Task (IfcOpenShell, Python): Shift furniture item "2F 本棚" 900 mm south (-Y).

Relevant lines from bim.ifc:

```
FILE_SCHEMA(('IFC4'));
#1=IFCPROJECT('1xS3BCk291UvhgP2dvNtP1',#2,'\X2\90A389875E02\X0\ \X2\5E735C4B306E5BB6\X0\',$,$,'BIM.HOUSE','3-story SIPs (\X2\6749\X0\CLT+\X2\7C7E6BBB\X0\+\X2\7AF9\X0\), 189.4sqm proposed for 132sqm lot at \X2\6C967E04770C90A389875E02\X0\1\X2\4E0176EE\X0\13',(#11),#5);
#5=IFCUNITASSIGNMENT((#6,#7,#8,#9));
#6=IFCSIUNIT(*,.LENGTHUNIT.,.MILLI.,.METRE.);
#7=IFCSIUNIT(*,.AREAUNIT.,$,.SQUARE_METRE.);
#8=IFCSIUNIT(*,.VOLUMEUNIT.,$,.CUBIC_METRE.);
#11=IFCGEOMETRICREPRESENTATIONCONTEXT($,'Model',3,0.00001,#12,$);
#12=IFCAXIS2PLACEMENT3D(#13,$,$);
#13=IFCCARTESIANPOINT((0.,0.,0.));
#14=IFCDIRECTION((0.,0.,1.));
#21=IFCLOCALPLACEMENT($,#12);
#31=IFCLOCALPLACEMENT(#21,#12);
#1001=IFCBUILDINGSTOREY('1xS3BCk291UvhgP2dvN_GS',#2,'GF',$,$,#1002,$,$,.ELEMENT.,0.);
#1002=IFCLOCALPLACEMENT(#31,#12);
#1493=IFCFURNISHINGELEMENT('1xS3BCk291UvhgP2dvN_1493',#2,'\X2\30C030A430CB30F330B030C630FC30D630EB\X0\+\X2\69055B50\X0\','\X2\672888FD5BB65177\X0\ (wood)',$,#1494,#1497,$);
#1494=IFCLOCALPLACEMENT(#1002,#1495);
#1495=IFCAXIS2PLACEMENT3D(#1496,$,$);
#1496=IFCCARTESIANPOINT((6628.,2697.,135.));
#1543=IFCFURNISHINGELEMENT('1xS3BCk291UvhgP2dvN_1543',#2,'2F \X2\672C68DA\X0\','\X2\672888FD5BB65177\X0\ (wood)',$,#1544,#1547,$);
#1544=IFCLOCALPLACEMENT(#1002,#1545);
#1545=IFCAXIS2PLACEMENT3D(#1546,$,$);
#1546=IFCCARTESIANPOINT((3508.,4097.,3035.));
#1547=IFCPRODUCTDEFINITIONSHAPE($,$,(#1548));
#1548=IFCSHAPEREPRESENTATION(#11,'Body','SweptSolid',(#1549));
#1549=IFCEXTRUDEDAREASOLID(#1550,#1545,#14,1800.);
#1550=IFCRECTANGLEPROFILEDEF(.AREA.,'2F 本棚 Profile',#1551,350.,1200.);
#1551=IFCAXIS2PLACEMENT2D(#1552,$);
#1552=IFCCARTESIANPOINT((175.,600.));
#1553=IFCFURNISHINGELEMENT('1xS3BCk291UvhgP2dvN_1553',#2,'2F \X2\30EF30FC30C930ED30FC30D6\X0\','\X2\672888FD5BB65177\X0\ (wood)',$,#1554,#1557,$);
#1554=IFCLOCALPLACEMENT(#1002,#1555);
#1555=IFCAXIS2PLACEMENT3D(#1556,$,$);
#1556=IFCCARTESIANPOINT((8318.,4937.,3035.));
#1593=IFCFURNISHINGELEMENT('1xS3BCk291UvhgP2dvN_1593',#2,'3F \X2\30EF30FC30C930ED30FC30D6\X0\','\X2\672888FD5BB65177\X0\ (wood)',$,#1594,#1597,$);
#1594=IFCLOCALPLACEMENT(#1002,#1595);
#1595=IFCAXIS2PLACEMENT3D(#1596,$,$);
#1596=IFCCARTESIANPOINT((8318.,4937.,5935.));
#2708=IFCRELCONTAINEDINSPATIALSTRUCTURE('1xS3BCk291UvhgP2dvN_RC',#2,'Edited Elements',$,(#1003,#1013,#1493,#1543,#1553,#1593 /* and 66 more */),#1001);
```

```python
import ifcopenshell
import ifcopenshell.api.geometry
import ifcopenshell.util.placement

model = ifcopenshell.open("bim.ifc")

item = model.by_guid("1xS3BCk291UvhgP2dvN_1543")
matrix = ifcopenshell.util.placement.get_local_placement(item.ObjectPlacement)
matrix[1, 3] -= 900.0
ifcopenshell.api.geometry.edit_object_placement(model, product=item, matrix=matrix, is_si=False)

print(ifcopenshell.util.placement.get_local_placement(item.ObjectPlacement).round(3) + 0.0)

model.write("bim_updated.ifc")
```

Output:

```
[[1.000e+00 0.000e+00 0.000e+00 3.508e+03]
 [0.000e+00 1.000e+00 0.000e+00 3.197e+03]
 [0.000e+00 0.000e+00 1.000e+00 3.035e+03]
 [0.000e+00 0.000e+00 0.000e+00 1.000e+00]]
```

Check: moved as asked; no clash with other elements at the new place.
